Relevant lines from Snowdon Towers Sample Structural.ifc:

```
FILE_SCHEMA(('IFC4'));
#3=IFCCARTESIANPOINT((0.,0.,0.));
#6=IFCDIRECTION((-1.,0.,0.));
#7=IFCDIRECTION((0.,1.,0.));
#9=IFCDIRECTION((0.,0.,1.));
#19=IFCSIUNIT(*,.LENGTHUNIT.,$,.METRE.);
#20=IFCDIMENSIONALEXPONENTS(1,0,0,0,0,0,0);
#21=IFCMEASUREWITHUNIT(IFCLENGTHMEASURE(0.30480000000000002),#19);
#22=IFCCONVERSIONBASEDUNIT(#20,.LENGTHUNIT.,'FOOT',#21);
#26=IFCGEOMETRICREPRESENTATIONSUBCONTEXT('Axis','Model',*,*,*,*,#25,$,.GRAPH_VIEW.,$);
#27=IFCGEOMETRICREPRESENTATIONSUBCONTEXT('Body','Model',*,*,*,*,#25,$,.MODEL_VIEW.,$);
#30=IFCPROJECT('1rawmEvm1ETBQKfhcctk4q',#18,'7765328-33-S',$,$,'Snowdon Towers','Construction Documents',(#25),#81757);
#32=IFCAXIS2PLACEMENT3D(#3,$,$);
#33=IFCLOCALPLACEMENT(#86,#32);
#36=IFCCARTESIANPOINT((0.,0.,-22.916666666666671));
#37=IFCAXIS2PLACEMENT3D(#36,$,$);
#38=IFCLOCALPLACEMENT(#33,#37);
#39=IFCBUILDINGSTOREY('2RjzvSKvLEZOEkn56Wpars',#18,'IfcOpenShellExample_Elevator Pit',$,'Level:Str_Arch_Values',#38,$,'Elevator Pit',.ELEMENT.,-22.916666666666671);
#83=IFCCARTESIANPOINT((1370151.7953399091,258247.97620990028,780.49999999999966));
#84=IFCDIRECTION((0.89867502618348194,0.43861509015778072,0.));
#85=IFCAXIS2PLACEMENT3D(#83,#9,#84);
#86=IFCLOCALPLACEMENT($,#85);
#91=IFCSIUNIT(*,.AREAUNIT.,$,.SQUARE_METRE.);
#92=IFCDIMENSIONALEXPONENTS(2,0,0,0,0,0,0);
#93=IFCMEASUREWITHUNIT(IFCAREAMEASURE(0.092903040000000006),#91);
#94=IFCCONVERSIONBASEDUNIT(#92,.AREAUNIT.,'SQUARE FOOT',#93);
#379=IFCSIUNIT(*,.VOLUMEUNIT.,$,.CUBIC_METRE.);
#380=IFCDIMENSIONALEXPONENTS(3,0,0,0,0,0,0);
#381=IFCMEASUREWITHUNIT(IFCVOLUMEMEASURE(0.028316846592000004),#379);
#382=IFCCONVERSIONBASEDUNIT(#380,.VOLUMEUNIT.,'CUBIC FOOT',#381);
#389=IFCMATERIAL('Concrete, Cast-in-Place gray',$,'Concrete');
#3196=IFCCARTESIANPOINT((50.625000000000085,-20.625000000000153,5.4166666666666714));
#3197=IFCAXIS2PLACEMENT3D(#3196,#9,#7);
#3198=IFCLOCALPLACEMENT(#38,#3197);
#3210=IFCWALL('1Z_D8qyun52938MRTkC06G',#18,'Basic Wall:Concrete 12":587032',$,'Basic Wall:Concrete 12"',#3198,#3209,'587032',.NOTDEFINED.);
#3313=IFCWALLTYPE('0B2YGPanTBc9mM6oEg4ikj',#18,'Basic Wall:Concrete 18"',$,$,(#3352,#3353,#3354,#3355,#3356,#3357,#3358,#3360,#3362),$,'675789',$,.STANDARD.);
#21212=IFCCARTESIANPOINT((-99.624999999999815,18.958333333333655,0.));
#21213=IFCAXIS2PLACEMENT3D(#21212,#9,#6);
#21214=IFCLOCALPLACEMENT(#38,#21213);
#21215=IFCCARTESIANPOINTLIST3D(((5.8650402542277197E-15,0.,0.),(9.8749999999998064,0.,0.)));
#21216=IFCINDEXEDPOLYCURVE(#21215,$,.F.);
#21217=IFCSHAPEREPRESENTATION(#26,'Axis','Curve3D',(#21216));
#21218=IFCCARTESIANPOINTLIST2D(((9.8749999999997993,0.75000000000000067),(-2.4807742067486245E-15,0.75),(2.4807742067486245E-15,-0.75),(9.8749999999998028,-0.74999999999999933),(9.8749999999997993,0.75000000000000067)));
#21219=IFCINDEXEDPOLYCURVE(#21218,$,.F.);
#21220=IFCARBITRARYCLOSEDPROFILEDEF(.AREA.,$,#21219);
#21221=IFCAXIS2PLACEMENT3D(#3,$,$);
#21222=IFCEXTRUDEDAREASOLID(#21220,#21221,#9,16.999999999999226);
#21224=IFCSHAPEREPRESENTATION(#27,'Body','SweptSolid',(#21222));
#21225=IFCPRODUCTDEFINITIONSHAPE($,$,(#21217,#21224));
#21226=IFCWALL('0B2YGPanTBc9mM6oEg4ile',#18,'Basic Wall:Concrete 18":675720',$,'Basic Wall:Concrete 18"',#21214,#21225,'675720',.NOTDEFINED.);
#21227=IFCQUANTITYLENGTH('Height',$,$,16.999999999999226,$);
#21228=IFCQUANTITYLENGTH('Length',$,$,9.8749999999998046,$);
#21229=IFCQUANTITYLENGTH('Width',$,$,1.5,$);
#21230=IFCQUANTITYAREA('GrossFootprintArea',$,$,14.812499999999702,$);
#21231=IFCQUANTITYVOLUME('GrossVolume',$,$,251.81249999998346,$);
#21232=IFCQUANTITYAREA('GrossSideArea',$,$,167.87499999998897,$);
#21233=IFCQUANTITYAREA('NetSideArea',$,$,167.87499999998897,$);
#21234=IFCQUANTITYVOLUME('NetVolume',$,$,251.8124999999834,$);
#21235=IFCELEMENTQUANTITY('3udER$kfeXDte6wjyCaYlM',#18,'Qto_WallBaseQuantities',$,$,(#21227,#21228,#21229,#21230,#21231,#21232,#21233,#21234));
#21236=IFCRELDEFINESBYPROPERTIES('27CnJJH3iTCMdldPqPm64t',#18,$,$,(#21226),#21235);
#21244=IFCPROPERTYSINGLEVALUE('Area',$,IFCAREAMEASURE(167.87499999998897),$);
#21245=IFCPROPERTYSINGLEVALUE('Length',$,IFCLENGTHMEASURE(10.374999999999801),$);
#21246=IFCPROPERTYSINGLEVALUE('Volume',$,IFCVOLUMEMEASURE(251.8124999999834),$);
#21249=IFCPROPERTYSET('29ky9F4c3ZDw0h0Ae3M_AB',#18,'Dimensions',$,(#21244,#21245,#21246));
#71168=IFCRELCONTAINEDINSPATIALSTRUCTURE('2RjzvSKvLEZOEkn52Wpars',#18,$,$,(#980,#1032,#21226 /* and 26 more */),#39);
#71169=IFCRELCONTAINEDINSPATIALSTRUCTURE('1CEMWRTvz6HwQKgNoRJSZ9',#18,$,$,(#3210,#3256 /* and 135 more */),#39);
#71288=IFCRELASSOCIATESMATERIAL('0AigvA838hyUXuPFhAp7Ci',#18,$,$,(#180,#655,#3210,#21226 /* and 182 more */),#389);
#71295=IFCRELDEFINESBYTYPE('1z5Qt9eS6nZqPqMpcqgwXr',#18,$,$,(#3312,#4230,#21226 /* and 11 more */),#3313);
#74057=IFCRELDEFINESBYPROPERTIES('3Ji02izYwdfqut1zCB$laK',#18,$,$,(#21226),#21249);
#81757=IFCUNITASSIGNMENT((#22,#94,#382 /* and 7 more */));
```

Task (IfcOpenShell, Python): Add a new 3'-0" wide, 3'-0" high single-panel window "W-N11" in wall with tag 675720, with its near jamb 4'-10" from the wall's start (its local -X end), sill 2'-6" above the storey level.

```python
import numpy as np
import ifcopenshell
import ifcopenshell.api.feature
import ifcopenshell.api.geometry
import ifcopenshell.api.pset
import ifcopenshell.api.root
import ifcopenshell.api.spatial
import ifcopenshell.geom
import ifcopenshell.util.element
import ifcopenshell.util.placement
import ifcopenshell.util.representation
import ifcopenshell.util.shape
import ifcopenshell.util.unit

model = ifcopenshell.open("Snowdon Towers Sample Structural.ifc")
unit_scale = ifcopenshell.util.unit.calculate_unit_scale(model)
area_scale = ifcopenshell.util.unit.calculate_unit_scale(model, "AREAUNIT")
volume_scale = ifcopenshell.util.unit.calculate_unit_scale(model, "VOLUMEUNIT")
settings = ifcopenshell.geom.settings()


def volume(element):
    """Net volume in cubic metres, openings subtracted."""
    shape = ifcopenshell.geom.create_shape(settings, element)
    return ifcopenshell.util.shape.get_volume(shape.geometry)


wall = model.by_id(21226)
storey = ifcopenshell.util.element.get_container(wall, ifc_class="IfcBuildingStorey")
context = ifcopenshell.util.representation.get_context(model, "Model", "Body", "MODEL_VIEW")
before = volume(wall)

width, height, from_end, sill = 0.9144, 0.9144, 1.4732, 0.762  # metres

# The wall runs along its own X axis, and the end named is its -X end.
wall_shape = ifcopenshell.geom.create_shape(settings, wall)
x, y, z = ifcopenshell.util.shape.get_vertices(wall_shape.geometry).T
start = x.min() + from_end
face, thickness = float(y.min()), float(y.max() - y.min())
wall_matrix = ifcopenshell.util.placement.get_local_placement(wall.ObjectPlacement)
level = ifcopenshell.util.placement.get_local_placement(storey.ObjectPlacement)[2, 3]


def in_wall(x, y):
    """Placement at x, y metres in the wall's axes, at sill height."""
    matrix = wall_matrix.copy()
    matrix[:, 3] = wall_matrix @ np.array([x / unit_scale, y / unit_scale, 0.0, 1.0])
    matrix[2, 3] = level + sill / unit_scale
    return matrix


# Opening: a box that overshoots both wall faces by 50 mm.
opening = ifcopenshell.api.root.create_entity(model, ifc_class="IfcOpeningElement", predefined_type="OPENING")
box = ifcopenshell.api.geometry.add_wall_representation(
    model, context=context, length=width, height=height, thickness=thickness + 0.1
)
ifcopenshell.api.geometry.assign_representation(model, product=opening, representation=box)
ifcopenshell.api.geometry.edit_object_placement(model, product=opening, matrix=in_wall(start, face - 0.05), is_si=False)
ifcopenshell.api.feature.add_feature(model, feature=opening, element=wall)

window = ifcopenshell.api.root.create_entity(model, ifc_class="IfcWindow", name="W-N11", predefined_type="WINDOW")
window.OverallWidth, window.OverallHeight = width / unit_scale, height / unit_scale
window.PartitioningType = "SINGLE_PANEL"
body = ifcopenshell.api.geometry.add_window_representation(
    model,
    context=context,
    overall_width=window.OverallWidth,
    overall_height=window.OverallHeight,
    partition_type="SINGLE_PANEL",
)
ifcopenshell.api.geometry.assign_representation(model, product=window, representation=body)
ifcopenshell.api.spatial.assign_container(model, products=[window], relating_structure=storey)
ifcopenshell.api.feature.add_filling(model, opening=opening, element=window)

# Centre the window in the wall's thickness.
ifcopenshell.api.geometry.edit_object_placement(model, product=window, matrix=in_wall(start, face), is_si=False)
window_shape = ifcopenshell.geom.create_shape(settings, window)
depth = ifcopenshell.util.shape.get_vertices(window_shape.geometry)[:, 1]
offset = face + thickness / 2 - (depth.min() + depth.max()) / 2
ifcopenshell.api.geometry.edit_object_placement(model, product=window, matrix=in_wall(start, offset), is_si=False)

after = volume(wall)

# Update the wall's stored quantities.
qto = model.by_id(ifcopenshell.util.element.get_pset(wall, "Qto_WallBaseQuantities", should_inherit=False)["id"])
ifcopenshell.api.pset.edit_qto(model, qto=qto, properties={
    "NetSideArea": after / thickness / area_scale,
    "NetVolume": after / volume_scale,
})
pset = model.by_id(ifcopenshell.util.element.get_pset(wall, "Dimensions", should_inherit=False)["id"])
ifcopenshell.api.pset.edit_pset(model, pset=pset, properties={
    "Area": model.create_entity("IfcAreaMeasure", after / thickness / area_scale),
    "Volume": model.create_entity("IfcVolumeMeasure", after / volume_scale),
})

print(f"wall volume {before:.3f} -> {after:.3f} m3")

model.write("Snowdon Towers Sample Structural_updated.ifc")
```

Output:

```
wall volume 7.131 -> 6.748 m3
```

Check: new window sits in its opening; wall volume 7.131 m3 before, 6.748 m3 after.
